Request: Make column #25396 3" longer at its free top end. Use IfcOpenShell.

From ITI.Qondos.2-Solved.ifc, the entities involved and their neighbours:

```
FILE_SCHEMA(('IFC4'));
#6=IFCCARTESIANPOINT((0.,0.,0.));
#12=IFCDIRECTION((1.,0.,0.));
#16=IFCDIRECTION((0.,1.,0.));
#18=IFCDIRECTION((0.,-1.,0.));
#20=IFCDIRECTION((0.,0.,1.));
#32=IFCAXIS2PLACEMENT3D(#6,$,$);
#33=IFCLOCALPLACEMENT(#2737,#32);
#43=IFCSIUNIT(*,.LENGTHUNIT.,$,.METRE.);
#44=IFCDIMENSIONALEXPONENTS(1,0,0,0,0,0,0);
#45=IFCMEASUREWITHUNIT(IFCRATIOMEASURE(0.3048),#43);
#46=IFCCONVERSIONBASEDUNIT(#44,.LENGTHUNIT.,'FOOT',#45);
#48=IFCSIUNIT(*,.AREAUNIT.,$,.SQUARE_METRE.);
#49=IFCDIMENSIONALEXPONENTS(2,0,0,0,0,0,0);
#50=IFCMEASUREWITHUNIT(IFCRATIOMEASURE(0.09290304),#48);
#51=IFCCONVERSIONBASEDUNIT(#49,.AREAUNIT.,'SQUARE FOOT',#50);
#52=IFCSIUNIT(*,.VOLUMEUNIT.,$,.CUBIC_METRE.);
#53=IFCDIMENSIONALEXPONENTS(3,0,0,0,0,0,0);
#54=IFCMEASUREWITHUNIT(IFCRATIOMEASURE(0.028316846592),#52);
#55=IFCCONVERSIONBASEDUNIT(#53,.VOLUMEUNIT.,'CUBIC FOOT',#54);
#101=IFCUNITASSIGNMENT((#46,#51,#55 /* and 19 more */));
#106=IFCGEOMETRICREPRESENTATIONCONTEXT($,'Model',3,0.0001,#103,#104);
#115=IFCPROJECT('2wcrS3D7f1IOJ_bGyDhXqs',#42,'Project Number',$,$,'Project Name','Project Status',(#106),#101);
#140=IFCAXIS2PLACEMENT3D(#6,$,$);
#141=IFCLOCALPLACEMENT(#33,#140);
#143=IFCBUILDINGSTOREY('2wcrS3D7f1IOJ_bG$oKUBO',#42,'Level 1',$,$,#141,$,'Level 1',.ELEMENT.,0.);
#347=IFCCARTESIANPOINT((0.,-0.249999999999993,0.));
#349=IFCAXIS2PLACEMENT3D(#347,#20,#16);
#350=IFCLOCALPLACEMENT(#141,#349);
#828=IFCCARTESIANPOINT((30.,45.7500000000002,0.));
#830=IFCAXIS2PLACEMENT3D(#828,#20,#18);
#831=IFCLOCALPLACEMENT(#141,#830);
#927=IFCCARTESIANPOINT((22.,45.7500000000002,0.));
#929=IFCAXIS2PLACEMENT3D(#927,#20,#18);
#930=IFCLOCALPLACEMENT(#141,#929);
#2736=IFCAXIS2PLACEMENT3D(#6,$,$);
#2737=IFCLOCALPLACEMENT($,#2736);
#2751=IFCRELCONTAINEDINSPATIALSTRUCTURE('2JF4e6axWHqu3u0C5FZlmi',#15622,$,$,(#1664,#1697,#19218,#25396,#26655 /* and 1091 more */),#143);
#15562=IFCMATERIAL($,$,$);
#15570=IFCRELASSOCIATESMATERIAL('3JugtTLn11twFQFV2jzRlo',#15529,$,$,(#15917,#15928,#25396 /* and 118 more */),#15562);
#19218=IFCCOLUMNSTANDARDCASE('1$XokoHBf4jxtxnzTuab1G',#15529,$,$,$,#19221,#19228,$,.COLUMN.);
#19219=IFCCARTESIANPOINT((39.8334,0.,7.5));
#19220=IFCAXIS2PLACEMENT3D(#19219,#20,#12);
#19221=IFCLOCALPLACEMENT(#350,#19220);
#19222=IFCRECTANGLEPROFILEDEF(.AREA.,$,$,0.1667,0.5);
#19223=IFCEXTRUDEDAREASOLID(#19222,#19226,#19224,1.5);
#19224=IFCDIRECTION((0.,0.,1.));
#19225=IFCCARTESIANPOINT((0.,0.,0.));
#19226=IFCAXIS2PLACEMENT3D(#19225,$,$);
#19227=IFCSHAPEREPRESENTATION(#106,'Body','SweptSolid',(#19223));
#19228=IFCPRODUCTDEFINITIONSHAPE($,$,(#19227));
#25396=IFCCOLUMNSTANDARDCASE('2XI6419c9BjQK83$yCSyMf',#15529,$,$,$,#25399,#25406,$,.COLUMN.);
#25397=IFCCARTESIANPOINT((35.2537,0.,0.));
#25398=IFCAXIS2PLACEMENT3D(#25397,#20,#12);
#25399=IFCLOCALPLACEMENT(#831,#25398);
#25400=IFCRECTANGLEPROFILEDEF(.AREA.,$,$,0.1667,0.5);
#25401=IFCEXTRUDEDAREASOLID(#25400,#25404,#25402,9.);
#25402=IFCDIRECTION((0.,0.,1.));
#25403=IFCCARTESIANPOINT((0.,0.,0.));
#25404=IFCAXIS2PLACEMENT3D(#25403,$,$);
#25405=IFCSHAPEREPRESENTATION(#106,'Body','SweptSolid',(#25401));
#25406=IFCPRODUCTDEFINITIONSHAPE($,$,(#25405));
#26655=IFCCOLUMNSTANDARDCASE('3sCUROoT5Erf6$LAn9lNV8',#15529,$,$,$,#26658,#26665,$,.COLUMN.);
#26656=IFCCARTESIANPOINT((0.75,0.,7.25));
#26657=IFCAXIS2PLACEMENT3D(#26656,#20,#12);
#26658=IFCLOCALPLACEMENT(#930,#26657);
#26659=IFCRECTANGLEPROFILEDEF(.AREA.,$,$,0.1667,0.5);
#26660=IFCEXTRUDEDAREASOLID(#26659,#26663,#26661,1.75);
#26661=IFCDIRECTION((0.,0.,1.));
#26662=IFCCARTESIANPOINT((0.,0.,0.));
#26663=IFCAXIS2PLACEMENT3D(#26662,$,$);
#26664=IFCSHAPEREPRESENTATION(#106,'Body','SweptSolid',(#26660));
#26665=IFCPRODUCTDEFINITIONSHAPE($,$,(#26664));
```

```python
import ifcopenshell
import ifcopenshell.util.unit

model = ifcopenshell.open("ITI.Qondos.2-Solved.ifc")
unit_scale = ifcopenshell.util.unit.calculate_unit_scale(model)

member = model.by_guid("2XI6419c9BjQK83$yCSyMf")
change = 3 * 0.0254 / unit_scale

# The extrusion runs towards the end named, so only its depth changes.
body = next(r for r in member.Representation.Representations if r.RepresentationIdentifier == "Body")
solid = body.Items[0]
old_length = solid.Depth
solid.Depth += change

print(f"length {old_length:g} -> {solid.Depth:g}")

model.write("ITI.Qondos.2-Solved_rev.ifc")
```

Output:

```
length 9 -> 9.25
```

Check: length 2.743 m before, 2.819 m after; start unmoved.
